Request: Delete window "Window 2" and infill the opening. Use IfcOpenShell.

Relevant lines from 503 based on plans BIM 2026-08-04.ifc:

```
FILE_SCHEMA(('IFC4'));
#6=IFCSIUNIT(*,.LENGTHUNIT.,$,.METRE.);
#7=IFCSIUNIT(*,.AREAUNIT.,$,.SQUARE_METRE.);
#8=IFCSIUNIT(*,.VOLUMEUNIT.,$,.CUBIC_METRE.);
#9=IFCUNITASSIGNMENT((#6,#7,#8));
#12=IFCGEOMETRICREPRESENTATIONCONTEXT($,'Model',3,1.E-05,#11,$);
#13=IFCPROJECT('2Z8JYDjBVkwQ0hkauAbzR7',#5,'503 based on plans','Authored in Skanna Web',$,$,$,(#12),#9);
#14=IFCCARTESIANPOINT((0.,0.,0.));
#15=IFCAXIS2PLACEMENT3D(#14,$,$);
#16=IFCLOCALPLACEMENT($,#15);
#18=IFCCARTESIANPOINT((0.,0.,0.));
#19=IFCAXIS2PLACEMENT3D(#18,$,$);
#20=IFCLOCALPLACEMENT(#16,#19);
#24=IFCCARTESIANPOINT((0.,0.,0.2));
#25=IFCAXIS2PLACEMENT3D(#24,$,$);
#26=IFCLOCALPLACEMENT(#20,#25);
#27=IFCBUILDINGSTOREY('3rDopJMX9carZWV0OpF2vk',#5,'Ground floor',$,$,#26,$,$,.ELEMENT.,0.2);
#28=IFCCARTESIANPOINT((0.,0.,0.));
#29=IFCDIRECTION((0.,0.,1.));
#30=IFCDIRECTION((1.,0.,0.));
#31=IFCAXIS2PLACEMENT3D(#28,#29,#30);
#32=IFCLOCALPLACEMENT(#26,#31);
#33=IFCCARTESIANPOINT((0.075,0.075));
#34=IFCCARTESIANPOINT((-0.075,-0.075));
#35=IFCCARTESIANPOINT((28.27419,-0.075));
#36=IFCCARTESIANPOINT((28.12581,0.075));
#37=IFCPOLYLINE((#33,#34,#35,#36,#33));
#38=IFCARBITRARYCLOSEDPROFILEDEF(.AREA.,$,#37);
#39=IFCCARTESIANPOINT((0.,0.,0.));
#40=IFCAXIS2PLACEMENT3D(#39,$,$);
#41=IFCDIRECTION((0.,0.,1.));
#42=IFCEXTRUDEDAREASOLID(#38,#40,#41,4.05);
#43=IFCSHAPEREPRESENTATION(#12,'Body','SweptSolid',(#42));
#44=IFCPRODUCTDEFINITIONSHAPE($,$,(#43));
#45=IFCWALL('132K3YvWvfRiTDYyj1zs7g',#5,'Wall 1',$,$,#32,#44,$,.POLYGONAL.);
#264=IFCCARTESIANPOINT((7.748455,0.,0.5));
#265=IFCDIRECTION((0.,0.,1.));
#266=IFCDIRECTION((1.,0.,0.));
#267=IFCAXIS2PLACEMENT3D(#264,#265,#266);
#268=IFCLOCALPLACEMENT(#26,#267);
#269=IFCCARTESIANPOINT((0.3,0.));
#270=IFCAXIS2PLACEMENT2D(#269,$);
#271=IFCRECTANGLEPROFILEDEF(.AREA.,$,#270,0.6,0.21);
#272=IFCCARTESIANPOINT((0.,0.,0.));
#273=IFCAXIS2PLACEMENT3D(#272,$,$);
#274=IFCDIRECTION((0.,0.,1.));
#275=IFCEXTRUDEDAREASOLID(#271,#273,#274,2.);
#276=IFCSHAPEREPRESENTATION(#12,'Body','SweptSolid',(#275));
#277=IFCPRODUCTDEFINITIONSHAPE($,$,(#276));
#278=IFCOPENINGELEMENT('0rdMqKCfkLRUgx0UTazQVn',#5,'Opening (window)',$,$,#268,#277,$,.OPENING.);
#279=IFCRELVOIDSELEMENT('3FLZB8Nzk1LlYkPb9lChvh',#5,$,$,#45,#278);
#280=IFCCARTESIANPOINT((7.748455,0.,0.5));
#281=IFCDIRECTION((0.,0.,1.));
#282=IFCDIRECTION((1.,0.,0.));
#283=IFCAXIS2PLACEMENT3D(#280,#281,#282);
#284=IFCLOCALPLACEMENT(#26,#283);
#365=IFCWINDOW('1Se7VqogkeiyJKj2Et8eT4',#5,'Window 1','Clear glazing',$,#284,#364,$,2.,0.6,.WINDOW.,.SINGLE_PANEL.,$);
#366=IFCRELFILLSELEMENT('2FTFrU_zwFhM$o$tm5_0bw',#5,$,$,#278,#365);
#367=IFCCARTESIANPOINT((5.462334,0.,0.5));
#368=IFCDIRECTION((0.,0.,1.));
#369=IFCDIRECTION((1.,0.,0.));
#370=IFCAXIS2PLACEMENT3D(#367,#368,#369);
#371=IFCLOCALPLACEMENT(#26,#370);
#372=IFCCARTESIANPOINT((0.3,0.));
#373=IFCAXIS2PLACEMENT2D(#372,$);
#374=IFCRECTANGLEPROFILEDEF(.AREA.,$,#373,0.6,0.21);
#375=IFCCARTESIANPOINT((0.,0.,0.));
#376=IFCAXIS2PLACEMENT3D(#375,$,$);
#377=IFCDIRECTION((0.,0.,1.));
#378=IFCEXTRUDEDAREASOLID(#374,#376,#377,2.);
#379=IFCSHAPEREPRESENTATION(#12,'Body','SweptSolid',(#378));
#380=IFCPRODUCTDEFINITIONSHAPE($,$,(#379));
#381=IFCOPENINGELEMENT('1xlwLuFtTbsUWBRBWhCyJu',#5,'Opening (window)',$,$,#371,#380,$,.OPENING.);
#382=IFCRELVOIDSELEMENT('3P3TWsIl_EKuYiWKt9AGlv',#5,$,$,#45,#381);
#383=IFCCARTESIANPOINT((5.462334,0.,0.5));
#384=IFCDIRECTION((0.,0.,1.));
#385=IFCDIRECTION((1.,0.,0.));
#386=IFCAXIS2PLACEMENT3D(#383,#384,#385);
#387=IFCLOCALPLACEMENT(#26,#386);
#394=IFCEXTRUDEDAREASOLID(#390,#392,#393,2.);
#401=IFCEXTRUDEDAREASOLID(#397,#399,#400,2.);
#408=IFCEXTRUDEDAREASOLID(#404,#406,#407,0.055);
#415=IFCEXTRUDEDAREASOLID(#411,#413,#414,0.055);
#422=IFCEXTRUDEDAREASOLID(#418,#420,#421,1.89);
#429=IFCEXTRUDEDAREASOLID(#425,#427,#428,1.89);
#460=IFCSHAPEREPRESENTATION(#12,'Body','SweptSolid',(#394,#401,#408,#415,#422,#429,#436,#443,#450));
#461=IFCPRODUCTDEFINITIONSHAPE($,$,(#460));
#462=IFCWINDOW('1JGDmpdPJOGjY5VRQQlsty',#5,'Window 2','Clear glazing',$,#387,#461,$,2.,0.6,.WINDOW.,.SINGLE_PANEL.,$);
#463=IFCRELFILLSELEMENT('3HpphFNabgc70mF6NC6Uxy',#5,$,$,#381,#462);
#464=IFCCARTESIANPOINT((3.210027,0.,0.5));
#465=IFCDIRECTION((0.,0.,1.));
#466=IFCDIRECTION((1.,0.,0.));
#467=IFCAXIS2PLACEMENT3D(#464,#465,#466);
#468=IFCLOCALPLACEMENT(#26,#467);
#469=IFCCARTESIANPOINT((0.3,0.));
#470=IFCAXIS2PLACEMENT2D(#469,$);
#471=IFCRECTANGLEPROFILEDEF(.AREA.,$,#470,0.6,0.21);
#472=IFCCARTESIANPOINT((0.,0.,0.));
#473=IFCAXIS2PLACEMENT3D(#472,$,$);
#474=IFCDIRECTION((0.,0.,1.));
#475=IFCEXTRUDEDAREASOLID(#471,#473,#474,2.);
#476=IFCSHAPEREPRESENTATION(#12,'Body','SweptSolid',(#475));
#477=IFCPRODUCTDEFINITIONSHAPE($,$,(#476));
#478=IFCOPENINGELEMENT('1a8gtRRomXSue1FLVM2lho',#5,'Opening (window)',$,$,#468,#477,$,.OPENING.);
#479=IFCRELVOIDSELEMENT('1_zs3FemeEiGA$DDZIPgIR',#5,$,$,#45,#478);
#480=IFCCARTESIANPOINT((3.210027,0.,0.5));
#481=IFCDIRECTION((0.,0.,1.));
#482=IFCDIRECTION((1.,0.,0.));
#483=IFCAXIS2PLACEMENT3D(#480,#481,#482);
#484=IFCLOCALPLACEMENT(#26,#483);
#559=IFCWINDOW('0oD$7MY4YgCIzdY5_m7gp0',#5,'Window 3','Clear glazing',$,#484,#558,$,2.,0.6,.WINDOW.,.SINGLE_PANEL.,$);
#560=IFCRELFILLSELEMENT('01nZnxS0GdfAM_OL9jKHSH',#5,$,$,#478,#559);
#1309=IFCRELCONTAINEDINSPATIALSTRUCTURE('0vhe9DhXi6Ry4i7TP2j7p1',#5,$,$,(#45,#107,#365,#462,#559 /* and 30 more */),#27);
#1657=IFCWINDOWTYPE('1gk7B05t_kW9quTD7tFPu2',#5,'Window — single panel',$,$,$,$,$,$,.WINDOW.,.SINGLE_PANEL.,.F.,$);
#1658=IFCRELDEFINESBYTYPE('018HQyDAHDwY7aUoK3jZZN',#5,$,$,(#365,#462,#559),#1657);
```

```python
import ifcopenshell
import ifcopenshell.api.feature
import ifcopenshell.api.root
import ifcopenshell.geom
import ifcopenshell.util.shape

model = ifcopenshell.open("503 based on plans BIM 2026-08-04.ifc")
settings = ifcopenshell.geom.settings()


def volume(element):
    """Net volume in cubic metres, openings subtracted."""
    shape = ifcopenshell.geom.create_shape(settings, element)
    return ifcopenshell.util.shape.get_volume(shape.geometry)


window = model.by_id(462)
opening = window.FillsVoids[0].RelatingOpeningElement
wall = opening.VoidsElements[0].RelatingBuildingElement
before = volume(wall)

ifcopenshell.api.root.remove_product(model, product=window)
ifcopenshell.api.feature.remove_feature(model, feature=opening)

after = volume(wall)

print(f"wall volume {before:.3f} -> {after:.3f} m3")

model.write("503 based on plans BIM 2026-08-04_rev.ifc")
```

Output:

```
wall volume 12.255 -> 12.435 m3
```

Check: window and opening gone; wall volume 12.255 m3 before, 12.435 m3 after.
